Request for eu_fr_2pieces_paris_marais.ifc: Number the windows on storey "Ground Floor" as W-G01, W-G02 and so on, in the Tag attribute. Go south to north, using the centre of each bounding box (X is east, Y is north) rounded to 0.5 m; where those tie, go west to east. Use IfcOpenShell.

First a look at what the model holds.

```python
import ifcopenshell
import ifcopenshell.util.element
import ifcopenshell.util.placement

model = ifcopenshell.open("eu_fr_2pieces_paris_marais.ifc")
print(model.schema)
storey = next(s for s in model.by_type("IfcBuildingStorey") if s.Name == "Ground Floor")
windows = [e for e in ifcopenshell.util.element.get_decomposition(storey) if e.is_a("IfcWindow")]
for e in sorted(windows, key=lambda e: e.id()):
    origin = ifcopenshell.util.placement.get_local_placement(e.ObjectPlacement)[:3, 3]
    print(e.id(), e.Tag, e.Name, origin.round(2) + 0.0, sep=" | ")
```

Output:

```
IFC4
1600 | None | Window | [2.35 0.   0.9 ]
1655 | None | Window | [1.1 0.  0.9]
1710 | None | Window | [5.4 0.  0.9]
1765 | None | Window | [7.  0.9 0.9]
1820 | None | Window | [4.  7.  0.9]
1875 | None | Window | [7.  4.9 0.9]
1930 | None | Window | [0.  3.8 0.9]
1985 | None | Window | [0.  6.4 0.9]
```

```python
import ifcopenshell
import ifcopenshell.geom
import ifcopenshell.util.element
import ifcopenshell.util.shape

model = ifcopenshell.open("eu_fr_2pieces_paris_marais.ifc")
settings = ifcopenshell.geom.settings()
settings.set("use-world-coords", True)


def centre(element):
    shape = ifcopenshell.geom.create_shape(settings, element)
    return ifcopenshell.util.shape.get_bbox_centroid(shape.geometry)


storey = next(s for s in model.by_type("IfcBuildingStorey") if s.Name == "Ground Floor")
windows = [e for e in ifcopenshell.util.element.get_decomposition(storey) if e.is_a("IfcWindow")]

# Insertion points can sit at a corner or the storey origin, so sort by the geometry (in metres).
centres = {e: centre(e) for e in windows}
windows.sort(key=lambda e: (round(centres[e][1] / 0.5), centres[e][0]))

for i, e in enumerate(windows, start=1):
    number = f"W-G{i:02d}"
    e.Tag = number
    print(e.id(), number)

model.write("eu_fr_2pieces_paris_marais-out.ifc")
```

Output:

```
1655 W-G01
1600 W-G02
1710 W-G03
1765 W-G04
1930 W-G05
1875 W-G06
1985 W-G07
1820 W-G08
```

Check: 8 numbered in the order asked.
